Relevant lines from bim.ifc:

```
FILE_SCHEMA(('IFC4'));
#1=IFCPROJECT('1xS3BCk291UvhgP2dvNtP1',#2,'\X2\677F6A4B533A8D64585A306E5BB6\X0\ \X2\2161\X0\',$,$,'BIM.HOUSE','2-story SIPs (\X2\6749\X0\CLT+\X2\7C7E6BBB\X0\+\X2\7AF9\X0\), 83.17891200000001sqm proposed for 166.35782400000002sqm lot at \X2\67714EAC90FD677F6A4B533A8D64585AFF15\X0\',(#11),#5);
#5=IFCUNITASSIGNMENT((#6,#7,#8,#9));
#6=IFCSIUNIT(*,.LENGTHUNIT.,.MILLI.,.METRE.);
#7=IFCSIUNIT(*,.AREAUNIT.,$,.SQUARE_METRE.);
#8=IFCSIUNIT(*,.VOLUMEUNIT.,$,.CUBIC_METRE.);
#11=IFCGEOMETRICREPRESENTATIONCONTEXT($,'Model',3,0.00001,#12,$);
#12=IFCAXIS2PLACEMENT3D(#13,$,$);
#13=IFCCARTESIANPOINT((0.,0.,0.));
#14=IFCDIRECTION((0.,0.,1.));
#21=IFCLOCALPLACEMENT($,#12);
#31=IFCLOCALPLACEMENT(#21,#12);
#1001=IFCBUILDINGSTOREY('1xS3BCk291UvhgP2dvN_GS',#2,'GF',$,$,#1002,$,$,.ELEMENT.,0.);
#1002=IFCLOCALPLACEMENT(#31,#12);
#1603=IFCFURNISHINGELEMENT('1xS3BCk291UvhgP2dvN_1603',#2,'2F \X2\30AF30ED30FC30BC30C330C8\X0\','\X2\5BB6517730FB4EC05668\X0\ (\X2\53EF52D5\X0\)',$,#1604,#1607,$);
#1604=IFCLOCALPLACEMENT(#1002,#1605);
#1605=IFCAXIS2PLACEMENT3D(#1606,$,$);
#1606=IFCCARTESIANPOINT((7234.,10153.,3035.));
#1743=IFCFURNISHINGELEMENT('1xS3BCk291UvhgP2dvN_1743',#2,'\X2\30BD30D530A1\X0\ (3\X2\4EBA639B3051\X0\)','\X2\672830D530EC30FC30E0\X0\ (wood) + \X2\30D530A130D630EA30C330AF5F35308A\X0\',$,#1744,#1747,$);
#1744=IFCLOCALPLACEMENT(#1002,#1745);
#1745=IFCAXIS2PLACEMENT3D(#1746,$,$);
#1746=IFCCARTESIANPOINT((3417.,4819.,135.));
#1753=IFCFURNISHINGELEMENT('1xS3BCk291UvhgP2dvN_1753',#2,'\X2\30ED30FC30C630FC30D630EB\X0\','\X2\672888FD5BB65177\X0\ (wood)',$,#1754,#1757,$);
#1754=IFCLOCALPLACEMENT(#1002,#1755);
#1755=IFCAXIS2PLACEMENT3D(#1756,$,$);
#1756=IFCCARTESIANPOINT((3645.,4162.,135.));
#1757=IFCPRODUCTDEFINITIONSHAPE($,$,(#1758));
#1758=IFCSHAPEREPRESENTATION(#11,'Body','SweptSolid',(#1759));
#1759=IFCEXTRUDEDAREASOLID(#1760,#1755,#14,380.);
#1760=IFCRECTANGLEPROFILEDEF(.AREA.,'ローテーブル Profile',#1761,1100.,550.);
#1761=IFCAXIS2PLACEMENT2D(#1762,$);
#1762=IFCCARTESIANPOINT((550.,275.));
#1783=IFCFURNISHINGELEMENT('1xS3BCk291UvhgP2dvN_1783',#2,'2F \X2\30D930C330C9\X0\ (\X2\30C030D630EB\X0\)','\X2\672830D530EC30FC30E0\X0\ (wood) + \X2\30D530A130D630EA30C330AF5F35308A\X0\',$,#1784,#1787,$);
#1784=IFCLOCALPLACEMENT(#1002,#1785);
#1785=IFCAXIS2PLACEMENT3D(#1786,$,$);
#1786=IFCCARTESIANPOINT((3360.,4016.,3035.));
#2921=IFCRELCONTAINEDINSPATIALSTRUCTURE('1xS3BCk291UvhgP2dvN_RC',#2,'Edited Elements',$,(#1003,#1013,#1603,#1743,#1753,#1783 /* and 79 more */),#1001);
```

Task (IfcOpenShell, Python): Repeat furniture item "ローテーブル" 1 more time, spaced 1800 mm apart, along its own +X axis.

```python
import ifcopenshell
import ifcopenshell.api.geometry
import ifcopenshell.api.root
import ifcopenshell.util.element
import ifcopenshell.util.placement

model = ifcopenshell.open("bim.ifc")


def reuse_history(source, copy):
    """copy_class also copies each property set's owner history, people and application; keep the originals."""
    for rel in copy.IsDefinedBy:
        if rel.is_a("IfcRelDefinesByProperties") and (history := rel.RelatingPropertyDefinition.OwnerHistory):
            rel.RelatingPropertyDefinition.OwnerHistory = source.OwnerHistory
            ifcopenshell.util.element.remove_deep2(model, history)


source = model.by_id(1753)
base = ifcopenshell.util.placement.get_local_placement(source.ObjectPlacement)
step = base[:3, 0] * 1800.0

for i in range(1, 2):
    copy = ifcopenshell.api.root.copy_class(model, product=source)
    copy.Representation = ifcopenshell.util.element.copy_deep(
        model, source.Representation, exclude=["IfcGeometricRepresentationContext", "IfcRepresentationMap"]
    )
    reuse_history(source, copy)
    matrix = base.copy()
    matrix[:3, 3] += i * step
    print("added at", matrix[:3, 3].round(3) + 0.0)
    ifcopenshell.api.geometry.edit_object_placement(model, product=copy, matrix=matrix, is_si=False)

model.write("bim-out.ifc")
```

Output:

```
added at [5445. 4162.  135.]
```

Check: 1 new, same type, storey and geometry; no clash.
